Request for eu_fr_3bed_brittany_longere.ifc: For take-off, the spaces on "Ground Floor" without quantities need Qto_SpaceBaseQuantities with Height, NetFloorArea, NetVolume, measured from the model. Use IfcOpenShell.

First a look at what the model holds.

```python
import ifcopenshell
import ifcopenshell.util.element
import ifcopenshell.util.unit

model = ifcopenshell.open("eu_fr_3bed_brittany_longere.ifc")
print(model.schema)
for unit_type in ("LENGTHUNIT", "AREAUNIT", "VOLUMEUNIT"):
    print(unit_type, ifcopenshell.util.unit.calculate_unit_scale(model, unit_type))
storey = next(s for s in model.by_type("IfcBuildingStorey") if s.Name == "Ground Floor")
spaces = [e for e in ifcopenshell.util.element.get_decomposition(storey) if e.is_a("IfcSpace")]
for e in sorted(spaces, key=lambda e: e.id()):
    print(e.id(), e.is_a(), e.Name, list(ifcopenshell.util.element.get_psets(e, qtos_only=True)), sep=" | ")
```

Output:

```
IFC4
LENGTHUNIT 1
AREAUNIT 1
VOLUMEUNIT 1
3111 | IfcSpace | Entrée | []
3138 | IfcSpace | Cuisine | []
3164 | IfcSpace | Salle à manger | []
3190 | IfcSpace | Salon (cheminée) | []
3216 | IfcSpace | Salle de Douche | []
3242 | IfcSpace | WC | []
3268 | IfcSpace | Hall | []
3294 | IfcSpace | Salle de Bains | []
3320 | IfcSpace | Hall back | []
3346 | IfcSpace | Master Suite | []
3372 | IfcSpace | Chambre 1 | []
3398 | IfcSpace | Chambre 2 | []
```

```python
import ifcopenshell
import ifcopenshell.api.pset
import ifcopenshell.geom
import ifcopenshell.util.element
import ifcopenshell.util.shape
import ifcopenshell.util.unit

model = ifcopenshell.open("eu_fr_3bed_brittany_longere.ifc")
unit_scale = ifcopenshell.util.unit.calculate_unit_scale(model)
area_scale = ifcopenshell.util.unit.calculate_unit_scale(model, "AREAUNIT")
volume_scale = ifcopenshell.util.unit.calculate_unit_scale(model, "VOLUMEUNIT")
settings = ifcopenshell.geom.settings()

storey = next(s for s in model.by_type("IfcBuildingStorey") if s.Name == "Ground Floor")
spaces = [e for e in ifcopenshell.util.element.get_decomposition(storey) if e.is_a("IfcSpace")]

for e in sorted(spaces, key=lambda e: e.id()):
    if ifcopenshell.util.element.get_psets(e, qtos_only=True, should_inherit=False):
        continue
    # Geometry comes back in metres, in the element's own axes.
    shape = ifcopenshell.geom.create_shape(settings, e)
    values = {
        "Height": ifcopenshell.util.shape.get_z(shape.geometry) / unit_scale,
        "NetFloorArea": ifcopenshell.util.shape.get_footprint_area(shape.geometry) / area_scale,
        "NetVolume": ifcopenshell.util.shape.get_volume(shape.geometry) / volume_scale,
    }
    qto = ifcopenshell.api.pset.add_qto(model, product=e, name="Qto_SpaceBaseQuantities")
    ifcopenshell.api.pset.edit_qto(model, qto=qto, properties=values)
    print(e.id(), {k: round(v, 3) for k, v in values.items()})

model.write("eu_fr_3bed_brittany_longere_updated.ifc")
```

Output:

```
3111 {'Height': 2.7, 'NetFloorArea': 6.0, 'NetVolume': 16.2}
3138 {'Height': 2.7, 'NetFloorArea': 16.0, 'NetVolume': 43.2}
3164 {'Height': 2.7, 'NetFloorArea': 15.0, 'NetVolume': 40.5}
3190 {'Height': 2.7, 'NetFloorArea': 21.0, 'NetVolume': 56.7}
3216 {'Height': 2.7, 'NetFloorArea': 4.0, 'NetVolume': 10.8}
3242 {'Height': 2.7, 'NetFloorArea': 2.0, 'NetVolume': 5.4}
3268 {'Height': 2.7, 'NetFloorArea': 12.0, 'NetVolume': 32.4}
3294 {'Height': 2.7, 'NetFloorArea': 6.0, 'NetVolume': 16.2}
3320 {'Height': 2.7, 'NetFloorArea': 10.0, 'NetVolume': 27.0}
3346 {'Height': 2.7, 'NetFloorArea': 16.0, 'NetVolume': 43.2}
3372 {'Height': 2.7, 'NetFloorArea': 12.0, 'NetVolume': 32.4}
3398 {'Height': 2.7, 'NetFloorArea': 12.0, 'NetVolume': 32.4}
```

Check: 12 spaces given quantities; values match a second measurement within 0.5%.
